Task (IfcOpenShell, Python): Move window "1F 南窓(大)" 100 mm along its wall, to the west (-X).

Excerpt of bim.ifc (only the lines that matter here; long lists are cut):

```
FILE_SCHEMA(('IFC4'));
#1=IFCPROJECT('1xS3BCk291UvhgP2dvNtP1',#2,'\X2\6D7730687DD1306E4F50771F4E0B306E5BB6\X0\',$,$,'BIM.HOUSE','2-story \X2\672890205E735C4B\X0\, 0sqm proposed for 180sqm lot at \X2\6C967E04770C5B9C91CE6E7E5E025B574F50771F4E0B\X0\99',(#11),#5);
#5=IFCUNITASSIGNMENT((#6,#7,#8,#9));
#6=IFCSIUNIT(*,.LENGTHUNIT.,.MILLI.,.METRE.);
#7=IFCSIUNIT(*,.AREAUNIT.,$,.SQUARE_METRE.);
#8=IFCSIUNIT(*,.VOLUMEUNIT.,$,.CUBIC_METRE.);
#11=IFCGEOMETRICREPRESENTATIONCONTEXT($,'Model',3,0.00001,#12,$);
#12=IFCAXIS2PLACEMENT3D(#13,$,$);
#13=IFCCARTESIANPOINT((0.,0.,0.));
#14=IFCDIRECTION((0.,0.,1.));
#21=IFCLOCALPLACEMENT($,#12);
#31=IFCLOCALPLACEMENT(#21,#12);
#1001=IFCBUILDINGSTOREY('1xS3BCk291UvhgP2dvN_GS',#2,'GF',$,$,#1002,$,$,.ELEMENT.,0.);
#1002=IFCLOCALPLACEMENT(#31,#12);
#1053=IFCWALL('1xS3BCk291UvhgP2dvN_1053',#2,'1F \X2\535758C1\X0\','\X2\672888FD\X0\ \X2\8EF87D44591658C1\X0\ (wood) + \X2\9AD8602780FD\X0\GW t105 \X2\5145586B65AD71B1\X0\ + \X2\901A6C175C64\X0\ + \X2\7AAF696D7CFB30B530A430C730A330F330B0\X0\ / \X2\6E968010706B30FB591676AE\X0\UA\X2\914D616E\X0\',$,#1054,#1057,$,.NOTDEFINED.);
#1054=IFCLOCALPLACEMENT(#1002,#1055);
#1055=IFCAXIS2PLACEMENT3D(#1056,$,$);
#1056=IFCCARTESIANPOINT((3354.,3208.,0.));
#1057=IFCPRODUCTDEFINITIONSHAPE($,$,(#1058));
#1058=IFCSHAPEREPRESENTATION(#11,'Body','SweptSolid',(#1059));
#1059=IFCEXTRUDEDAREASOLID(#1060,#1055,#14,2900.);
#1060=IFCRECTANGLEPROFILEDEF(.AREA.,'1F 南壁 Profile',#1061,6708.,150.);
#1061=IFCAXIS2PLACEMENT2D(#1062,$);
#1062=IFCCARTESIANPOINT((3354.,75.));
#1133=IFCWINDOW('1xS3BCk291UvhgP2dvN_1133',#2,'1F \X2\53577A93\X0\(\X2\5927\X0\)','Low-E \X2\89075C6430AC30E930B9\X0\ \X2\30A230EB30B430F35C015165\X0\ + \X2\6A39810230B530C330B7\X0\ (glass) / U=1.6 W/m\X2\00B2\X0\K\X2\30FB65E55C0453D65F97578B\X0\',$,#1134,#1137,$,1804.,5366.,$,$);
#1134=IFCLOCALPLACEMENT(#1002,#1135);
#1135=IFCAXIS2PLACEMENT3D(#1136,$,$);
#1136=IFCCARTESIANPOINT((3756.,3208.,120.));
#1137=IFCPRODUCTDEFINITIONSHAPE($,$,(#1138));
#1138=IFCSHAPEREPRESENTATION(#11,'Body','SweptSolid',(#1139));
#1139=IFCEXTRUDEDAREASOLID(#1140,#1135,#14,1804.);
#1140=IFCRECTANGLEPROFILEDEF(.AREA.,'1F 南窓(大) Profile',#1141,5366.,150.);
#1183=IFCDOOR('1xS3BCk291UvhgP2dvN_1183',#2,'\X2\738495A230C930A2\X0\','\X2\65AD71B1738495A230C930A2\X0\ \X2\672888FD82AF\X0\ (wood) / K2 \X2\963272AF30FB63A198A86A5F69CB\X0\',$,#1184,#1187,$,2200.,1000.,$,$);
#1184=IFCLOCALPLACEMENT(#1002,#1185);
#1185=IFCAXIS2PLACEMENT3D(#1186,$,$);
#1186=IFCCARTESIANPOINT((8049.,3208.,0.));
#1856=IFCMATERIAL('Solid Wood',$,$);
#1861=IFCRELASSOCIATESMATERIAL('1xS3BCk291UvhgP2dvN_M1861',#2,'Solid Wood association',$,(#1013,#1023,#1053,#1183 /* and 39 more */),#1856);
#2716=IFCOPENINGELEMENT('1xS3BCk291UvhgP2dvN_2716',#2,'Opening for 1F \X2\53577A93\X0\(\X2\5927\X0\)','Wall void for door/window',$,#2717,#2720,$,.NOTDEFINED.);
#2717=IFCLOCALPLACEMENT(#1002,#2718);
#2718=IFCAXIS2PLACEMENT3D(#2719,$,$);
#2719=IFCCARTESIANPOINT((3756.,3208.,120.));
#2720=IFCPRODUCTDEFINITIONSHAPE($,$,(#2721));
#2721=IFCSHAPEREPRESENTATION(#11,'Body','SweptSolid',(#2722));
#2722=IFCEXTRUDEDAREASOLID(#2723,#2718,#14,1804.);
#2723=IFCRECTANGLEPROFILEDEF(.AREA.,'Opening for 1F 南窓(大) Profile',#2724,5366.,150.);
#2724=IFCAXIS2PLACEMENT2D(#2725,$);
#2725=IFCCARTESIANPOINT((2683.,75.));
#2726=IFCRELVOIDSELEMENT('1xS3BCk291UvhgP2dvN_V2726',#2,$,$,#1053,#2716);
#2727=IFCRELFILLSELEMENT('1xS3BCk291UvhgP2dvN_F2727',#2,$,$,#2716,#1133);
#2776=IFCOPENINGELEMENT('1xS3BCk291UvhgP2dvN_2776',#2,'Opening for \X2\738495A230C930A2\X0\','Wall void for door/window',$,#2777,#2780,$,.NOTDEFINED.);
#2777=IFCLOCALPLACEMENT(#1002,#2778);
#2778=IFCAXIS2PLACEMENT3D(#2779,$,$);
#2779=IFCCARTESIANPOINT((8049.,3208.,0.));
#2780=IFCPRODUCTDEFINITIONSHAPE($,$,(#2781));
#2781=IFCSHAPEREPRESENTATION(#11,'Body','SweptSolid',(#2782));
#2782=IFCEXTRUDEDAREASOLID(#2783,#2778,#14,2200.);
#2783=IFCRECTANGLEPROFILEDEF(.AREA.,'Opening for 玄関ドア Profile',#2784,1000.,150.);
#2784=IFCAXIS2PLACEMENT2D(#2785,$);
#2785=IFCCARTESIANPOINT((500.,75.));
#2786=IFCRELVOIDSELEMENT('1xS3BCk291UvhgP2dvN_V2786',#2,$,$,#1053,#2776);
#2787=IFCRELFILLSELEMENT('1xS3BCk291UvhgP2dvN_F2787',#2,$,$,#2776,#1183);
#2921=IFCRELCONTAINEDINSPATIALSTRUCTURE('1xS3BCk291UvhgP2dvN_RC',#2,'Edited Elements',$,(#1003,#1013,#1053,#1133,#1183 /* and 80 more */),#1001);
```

```python
import ifcopenshell
import ifcopenshell.api.geometry
import ifcopenshell.util.placement
import ifcopenshell.util.unit

model = ifcopenshell.open("bim.ifc")
unit_scale = ifcopenshell.util.unit.calculate_unit_scale(model)

window = model.by_guid("1xS3BCk291UvhgP2dvN_1133")
opening = window.FillsVoids[0].RelatingOpeningElement
wall = opening.VoidsElements[0].RelatingBuildingElement

wall_matrix = ifcopenshell.util.placement.get_local_placement(wall.ObjectPlacement)
shift = wall_matrix[:3, 0] * -0.1 / unit_scale
before = ifcopenshell.util.placement.get_local_placement(window.ObjectPlacement)[:3, 3].copy()

# The window is not placed relative to its opening, so move both.
for product in (opening, window):
    matrix = ifcopenshell.util.placement.get_local_placement(product.ObjectPlacement)
    matrix[:3, 3] += shift
    ifcopenshell.api.geometry.edit_object_placement(model, product=product, matrix=matrix, is_si=False)

after = ifcopenshell.util.placement.get_local_placement(window.ObjectPlacement)[:3, 3]
print("window moved by", (after - before).round(3) + 0.0)

model.write("bim_v2.ifc")
```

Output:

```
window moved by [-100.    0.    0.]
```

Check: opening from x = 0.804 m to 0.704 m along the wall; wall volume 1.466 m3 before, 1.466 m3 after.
